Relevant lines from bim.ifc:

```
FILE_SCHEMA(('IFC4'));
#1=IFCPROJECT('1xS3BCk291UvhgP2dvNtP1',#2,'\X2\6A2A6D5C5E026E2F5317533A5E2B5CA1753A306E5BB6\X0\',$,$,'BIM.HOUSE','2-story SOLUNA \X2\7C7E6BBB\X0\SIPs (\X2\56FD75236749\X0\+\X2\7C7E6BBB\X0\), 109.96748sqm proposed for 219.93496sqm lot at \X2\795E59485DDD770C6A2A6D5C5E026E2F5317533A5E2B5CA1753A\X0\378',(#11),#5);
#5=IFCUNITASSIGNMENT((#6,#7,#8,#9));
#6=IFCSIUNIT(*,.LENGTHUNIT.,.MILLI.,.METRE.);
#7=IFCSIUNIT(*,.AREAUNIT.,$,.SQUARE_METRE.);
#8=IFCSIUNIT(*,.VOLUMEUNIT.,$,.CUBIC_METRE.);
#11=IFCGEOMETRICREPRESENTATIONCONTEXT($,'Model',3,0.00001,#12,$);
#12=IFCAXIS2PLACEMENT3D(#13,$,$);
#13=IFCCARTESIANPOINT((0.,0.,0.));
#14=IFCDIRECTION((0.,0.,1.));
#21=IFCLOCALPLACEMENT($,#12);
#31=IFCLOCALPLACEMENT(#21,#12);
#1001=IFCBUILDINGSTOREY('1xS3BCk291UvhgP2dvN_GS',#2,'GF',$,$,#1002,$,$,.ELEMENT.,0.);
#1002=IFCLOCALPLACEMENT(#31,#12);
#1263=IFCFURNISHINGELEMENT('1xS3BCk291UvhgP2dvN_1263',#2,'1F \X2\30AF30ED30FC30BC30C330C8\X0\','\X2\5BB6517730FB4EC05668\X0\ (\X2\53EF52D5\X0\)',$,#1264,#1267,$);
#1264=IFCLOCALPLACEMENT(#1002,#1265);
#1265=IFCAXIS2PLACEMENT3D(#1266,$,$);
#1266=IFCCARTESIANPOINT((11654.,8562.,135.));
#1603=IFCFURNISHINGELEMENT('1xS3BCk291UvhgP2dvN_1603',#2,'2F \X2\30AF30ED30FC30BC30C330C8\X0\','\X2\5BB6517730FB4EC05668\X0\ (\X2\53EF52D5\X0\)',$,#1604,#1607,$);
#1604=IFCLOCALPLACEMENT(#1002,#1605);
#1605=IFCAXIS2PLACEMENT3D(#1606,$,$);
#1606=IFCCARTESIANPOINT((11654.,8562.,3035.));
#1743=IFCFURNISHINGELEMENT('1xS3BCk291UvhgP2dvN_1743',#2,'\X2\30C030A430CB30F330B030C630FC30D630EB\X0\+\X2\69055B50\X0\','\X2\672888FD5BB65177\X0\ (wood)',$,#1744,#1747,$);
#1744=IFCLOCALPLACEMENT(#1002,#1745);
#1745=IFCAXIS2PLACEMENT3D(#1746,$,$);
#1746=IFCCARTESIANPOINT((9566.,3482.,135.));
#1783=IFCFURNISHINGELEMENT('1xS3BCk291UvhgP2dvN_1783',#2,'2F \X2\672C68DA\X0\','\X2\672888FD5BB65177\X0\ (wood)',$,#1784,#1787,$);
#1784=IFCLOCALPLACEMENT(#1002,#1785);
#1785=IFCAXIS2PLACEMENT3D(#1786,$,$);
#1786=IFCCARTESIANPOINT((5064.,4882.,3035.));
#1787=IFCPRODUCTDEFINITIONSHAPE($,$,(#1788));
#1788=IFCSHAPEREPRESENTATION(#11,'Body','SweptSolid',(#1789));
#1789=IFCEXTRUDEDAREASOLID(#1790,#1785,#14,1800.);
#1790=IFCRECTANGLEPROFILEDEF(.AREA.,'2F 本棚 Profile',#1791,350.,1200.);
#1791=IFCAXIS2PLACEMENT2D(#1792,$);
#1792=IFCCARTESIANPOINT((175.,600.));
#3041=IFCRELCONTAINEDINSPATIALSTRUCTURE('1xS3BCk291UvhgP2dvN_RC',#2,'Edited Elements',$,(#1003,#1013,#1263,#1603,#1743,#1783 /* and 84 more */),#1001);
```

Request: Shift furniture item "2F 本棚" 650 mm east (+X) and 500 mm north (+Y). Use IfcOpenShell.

```python
import ifcopenshell
import ifcopenshell.api.geometry
import ifcopenshell.util.placement

model = ifcopenshell.open("bim.ifc")

item = model.by_guid("1xS3BCk291UvhgP2dvN_1783")
matrix = ifcopenshell.util.placement.get_local_placement(item.ObjectPlacement)
matrix[0, 3] += 650.0
matrix[1, 3] += 500.0
ifcopenshell.api.geometry.edit_object_placement(model, product=item, matrix=matrix, is_si=False)

print(ifcopenshell.util.placement.get_local_placement(item.ObjectPlacement).round(3) + 0.0)

model.write("bim_rev.ifc")
```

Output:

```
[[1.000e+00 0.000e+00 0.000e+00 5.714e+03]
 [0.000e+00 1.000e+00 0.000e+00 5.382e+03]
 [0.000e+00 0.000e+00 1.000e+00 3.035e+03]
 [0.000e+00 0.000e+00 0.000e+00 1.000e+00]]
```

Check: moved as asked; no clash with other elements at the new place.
